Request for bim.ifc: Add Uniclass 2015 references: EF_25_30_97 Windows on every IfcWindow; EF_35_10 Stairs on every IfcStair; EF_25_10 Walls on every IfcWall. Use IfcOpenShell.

First a look at what the model holds.

```python
import ifcopenshell

model = ifcopenshell.open("bim.ifc")
print(model.schema)
print("classifications:", [c.Name for c in model.by_type("IfcClassification")])
for ifc_class in ("IfcDoor", "IfcRoof", "IfcStair", "IfcWall", "IfcWindow"):
    print(ifc_class, len(model.by_type(ifc_class)))
```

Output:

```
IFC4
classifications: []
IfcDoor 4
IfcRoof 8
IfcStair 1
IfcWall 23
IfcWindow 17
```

```python
import ifcopenshell
import ifcopenshell.api.classification

model = ifcopenshell.open("bim.ifc")

system = ifcopenshell.api.classification.add_classification(model, classification="Uniclass 2015")

codes = {
    "IfcWindow": ("EF_25_30_97", "Windows"),
    "IfcStair": ("EF_35_10", "Stairs"),
    "IfcWall": ("EF_25_10", "Walls"),
}
for ifc_class, (code, name) in codes.items():
    products = model.by_type(ifc_class)
    ifcopenshell.api.classification.add_reference(
        model, products=products, classification=system, identification=code, name=name
    )
    print(code, len(products))

model.write("bim_rev.ifc")
```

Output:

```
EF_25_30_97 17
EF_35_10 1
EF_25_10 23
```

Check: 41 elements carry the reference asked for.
